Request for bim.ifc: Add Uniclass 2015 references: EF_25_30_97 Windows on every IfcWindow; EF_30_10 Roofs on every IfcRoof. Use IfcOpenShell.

First a look at what the model holds.

```python
import ifcopenshell

model = ifcopenshell.open("bim.ifc")
print(model.schema)
print("classifications:", [c.Name for c in model.by_type("IfcClassification")])
for ifc_class in ("IfcDoor", "IfcRoof", "IfcStair", "IfcWall", "IfcWindow"):
    print(ifc_class, len(model.by_type(ifc_class)))
```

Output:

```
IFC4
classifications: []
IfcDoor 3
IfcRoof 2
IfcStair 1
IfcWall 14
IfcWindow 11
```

```python
import ifcopenshell
import ifcopenshell.api.classification

model = ifcopenshell.open("bim.ifc")

system = ifcopenshell.api.classification.add_classification(model, classification="Uniclass 2015")

codes = {
    "IfcWindow": ("EF_25_30_97", "Windows"),
    "IfcRoof": ("EF_30_10", "Roofs"),
}
for ifc_class, (code, name) in codes.items():
    products = model.by_type(ifc_class)
    ifcopenshell.api.classification.add_reference(
        model, products=products, classification=system, identification=code, name=name
    )
    print(code, len(products))

model.write("bim_edited.ifc")
```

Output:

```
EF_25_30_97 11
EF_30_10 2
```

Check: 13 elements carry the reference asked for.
